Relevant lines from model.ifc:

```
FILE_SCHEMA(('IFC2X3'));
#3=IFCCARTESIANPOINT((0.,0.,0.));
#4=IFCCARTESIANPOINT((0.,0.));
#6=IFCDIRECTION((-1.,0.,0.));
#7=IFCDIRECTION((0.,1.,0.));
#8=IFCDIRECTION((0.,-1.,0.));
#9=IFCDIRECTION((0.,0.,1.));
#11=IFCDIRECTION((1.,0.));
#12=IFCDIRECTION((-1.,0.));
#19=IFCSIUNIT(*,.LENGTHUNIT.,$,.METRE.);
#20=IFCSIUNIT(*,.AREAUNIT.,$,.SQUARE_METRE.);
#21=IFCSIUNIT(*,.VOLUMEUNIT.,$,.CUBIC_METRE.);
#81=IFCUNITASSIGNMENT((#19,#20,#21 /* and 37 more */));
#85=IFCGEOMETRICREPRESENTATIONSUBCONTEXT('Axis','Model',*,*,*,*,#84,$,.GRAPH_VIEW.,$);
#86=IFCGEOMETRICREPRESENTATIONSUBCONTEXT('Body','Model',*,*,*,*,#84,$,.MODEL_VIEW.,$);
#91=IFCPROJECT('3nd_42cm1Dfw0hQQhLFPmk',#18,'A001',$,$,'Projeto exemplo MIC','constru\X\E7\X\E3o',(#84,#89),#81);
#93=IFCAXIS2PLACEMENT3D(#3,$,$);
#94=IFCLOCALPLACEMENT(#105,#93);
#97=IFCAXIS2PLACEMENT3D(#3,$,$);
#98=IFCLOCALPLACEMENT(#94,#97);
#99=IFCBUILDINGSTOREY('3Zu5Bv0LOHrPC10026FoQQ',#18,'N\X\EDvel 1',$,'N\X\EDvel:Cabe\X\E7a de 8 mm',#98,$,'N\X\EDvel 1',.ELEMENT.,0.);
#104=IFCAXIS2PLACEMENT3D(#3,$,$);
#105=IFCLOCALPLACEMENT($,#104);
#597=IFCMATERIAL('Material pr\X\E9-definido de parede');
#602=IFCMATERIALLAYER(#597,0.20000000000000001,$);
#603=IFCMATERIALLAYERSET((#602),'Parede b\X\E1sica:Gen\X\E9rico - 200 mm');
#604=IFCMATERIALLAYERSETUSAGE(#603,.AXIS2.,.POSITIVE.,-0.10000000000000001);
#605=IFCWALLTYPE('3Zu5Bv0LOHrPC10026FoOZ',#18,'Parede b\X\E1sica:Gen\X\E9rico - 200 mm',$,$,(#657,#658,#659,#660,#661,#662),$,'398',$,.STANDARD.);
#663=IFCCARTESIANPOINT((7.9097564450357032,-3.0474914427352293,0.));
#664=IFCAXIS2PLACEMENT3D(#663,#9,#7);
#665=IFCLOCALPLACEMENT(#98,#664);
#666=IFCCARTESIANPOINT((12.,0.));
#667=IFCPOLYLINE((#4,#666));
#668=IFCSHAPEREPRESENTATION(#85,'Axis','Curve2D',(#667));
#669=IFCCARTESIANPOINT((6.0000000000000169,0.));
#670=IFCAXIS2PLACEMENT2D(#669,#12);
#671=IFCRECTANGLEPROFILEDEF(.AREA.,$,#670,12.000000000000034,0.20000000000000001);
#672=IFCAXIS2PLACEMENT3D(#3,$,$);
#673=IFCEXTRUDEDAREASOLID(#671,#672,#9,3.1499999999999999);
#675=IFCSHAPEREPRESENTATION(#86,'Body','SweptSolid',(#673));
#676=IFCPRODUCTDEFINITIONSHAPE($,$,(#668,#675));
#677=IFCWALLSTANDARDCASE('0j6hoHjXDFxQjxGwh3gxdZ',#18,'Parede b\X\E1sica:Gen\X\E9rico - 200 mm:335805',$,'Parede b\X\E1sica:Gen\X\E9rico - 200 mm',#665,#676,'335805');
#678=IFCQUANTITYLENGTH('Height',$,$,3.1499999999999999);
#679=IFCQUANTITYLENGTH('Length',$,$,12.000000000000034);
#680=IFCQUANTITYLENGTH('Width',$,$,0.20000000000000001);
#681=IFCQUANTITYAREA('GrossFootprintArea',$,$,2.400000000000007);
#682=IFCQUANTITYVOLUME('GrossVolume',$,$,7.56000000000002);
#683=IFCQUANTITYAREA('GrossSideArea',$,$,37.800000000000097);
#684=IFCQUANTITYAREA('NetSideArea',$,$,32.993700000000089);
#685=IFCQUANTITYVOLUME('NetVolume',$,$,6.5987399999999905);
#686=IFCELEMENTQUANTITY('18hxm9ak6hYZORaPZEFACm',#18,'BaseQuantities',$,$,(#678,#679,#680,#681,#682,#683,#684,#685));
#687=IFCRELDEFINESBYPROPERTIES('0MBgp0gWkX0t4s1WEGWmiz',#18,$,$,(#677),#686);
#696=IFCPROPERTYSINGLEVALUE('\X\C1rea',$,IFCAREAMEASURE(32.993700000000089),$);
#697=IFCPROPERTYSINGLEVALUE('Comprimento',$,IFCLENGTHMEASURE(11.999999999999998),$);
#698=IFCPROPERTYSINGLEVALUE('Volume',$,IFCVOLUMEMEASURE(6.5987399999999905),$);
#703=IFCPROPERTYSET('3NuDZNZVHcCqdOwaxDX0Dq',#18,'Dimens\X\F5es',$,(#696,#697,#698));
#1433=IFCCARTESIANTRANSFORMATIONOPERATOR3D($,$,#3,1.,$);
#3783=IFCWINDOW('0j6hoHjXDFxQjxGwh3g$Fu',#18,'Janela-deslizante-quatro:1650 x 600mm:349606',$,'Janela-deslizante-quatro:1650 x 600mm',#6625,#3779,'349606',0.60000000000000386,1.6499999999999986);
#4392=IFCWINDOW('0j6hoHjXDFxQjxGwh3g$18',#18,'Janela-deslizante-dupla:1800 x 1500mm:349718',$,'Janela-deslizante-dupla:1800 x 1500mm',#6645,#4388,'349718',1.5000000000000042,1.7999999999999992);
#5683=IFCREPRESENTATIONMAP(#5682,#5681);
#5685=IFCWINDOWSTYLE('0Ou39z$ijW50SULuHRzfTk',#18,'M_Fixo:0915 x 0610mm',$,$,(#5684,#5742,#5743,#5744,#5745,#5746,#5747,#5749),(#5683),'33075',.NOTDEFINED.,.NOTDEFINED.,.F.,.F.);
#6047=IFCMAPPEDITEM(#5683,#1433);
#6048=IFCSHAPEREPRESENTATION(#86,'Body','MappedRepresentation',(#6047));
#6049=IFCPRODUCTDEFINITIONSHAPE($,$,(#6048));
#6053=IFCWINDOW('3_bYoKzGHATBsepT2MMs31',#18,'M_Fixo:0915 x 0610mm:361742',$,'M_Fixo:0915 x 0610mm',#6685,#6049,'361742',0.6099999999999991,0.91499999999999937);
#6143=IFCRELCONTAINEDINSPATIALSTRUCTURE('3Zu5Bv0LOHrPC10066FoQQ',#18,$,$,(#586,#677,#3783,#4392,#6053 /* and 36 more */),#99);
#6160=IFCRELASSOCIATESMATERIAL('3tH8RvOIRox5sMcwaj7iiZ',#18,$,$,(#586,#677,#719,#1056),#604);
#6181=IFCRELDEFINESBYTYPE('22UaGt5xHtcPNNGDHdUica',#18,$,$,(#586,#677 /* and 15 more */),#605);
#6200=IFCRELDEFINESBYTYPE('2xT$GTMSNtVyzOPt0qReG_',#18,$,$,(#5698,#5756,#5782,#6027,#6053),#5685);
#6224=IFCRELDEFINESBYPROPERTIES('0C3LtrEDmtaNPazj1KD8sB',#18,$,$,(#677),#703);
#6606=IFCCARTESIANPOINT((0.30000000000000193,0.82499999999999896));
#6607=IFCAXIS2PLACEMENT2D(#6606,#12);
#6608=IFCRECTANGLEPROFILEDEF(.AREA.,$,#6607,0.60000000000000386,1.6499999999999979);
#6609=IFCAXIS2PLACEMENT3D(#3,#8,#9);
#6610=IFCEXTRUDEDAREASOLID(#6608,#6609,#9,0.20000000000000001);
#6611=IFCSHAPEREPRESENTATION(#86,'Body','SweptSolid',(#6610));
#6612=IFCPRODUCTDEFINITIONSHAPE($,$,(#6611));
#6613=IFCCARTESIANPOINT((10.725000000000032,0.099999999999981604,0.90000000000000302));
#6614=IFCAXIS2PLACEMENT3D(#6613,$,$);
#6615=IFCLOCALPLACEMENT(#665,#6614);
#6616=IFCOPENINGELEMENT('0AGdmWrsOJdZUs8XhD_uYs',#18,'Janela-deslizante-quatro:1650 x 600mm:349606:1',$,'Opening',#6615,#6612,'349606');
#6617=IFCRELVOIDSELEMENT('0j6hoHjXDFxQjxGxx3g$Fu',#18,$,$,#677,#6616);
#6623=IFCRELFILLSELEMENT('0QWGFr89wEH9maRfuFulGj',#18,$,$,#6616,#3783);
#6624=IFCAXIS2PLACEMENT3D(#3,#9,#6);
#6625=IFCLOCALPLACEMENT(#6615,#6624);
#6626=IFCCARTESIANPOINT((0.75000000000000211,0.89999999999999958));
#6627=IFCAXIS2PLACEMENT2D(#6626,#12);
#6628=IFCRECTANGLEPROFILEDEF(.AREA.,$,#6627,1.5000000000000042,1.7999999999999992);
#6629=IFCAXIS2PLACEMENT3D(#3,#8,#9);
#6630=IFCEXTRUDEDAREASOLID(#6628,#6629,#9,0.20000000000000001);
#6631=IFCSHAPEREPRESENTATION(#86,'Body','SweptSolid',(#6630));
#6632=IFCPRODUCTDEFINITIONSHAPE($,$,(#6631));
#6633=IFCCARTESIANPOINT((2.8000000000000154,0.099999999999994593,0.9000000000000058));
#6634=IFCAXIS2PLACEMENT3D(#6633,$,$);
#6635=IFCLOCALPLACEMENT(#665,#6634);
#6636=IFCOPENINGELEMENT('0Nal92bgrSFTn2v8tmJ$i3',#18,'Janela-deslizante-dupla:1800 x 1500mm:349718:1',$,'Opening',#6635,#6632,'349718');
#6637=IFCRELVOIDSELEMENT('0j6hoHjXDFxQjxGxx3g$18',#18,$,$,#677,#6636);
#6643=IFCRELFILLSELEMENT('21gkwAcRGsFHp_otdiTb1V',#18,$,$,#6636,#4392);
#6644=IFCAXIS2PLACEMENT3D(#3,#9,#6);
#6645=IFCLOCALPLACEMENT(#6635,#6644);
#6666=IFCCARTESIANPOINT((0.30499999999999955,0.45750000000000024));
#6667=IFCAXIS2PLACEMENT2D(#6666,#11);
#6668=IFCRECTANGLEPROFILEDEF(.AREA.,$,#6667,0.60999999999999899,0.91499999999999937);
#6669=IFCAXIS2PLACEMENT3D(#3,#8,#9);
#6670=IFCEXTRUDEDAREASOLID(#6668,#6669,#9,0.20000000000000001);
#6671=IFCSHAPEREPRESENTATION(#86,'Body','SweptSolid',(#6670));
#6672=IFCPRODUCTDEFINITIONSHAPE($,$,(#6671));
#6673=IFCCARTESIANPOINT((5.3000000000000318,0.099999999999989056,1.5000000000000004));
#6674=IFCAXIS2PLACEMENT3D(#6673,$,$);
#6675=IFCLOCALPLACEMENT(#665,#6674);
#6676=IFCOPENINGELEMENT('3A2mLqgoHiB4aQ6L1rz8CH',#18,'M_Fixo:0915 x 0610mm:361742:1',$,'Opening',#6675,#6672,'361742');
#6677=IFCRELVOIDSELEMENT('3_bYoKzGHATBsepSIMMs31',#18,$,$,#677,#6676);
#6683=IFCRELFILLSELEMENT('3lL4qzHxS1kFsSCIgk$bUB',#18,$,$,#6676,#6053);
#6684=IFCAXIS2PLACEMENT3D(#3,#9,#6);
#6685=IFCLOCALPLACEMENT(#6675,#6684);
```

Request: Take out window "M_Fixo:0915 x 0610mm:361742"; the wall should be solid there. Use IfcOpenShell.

```python
import ifcopenshell
import ifcopenshell.api.feature
import ifcopenshell.api.pset
import ifcopenshell.api.root
import ifcopenshell.geom
import ifcopenshell.util.element
import ifcopenshell.util.shape
import ifcopenshell.util.unit

model = ifcopenshell.open("model.ifc")
area_scale = ifcopenshell.util.unit.calculate_unit_scale(model, "AREAUNIT")
volume_scale = ifcopenshell.util.unit.calculate_unit_scale(model, "VOLUMEUNIT")
settings = ifcopenshell.geom.settings()


def volume(element):
    """Net volume in cubic metres, openings subtracted."""
    shape = ifcopenshell.geom.create_shape(settings, element)
    return ifcopenshell.util.shape.get_volume(shape.geometry)


window = model.by_id(6053)
opening = window.FillsVoids[0].RelatingOpeningElement
wall = opening.VoidsElements[0].RelatingBuildingElement
before = volume(wall)

ifcopenshell.api.root.remove_product(model, product=window)
ifcopenshell.api.feature.remove_feature(model, feature=opening)

after = volume(wall)
thickness = 0.2  # wall thickness in metres

# Update the wall's stored quantities.
qto = model.by_id(ifcopenshell.util.element.get_pset(wall, "BaseQuantities", should_inherit=False)["id"])
ifcopenshell.api.pset.edit_qto(model, qto=qto, properties={
    "NetSideArea": after / thickness / area_scale,
    "NetVolume": after / volume_scale,
})
pset = model.by_id(ifcopenshell.util.element.get_pset(wall, "Dimensões", should_inherit=False)["id"])
ifcopenshell.api.pset.edit_pset(model, pset=pset, properties={
    "Área": model.create_entity("IfcAreaMeasure", after / thickness / area_scale),
    "Volume": model.create_entity("IfcVolumeMeasure", after / volume_scale),
})

print(f"wall volume {before:.3f} -> {after:.3f} m3")

model.write("model_edited.ifc")
```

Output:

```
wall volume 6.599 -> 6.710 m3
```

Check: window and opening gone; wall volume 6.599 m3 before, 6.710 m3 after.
